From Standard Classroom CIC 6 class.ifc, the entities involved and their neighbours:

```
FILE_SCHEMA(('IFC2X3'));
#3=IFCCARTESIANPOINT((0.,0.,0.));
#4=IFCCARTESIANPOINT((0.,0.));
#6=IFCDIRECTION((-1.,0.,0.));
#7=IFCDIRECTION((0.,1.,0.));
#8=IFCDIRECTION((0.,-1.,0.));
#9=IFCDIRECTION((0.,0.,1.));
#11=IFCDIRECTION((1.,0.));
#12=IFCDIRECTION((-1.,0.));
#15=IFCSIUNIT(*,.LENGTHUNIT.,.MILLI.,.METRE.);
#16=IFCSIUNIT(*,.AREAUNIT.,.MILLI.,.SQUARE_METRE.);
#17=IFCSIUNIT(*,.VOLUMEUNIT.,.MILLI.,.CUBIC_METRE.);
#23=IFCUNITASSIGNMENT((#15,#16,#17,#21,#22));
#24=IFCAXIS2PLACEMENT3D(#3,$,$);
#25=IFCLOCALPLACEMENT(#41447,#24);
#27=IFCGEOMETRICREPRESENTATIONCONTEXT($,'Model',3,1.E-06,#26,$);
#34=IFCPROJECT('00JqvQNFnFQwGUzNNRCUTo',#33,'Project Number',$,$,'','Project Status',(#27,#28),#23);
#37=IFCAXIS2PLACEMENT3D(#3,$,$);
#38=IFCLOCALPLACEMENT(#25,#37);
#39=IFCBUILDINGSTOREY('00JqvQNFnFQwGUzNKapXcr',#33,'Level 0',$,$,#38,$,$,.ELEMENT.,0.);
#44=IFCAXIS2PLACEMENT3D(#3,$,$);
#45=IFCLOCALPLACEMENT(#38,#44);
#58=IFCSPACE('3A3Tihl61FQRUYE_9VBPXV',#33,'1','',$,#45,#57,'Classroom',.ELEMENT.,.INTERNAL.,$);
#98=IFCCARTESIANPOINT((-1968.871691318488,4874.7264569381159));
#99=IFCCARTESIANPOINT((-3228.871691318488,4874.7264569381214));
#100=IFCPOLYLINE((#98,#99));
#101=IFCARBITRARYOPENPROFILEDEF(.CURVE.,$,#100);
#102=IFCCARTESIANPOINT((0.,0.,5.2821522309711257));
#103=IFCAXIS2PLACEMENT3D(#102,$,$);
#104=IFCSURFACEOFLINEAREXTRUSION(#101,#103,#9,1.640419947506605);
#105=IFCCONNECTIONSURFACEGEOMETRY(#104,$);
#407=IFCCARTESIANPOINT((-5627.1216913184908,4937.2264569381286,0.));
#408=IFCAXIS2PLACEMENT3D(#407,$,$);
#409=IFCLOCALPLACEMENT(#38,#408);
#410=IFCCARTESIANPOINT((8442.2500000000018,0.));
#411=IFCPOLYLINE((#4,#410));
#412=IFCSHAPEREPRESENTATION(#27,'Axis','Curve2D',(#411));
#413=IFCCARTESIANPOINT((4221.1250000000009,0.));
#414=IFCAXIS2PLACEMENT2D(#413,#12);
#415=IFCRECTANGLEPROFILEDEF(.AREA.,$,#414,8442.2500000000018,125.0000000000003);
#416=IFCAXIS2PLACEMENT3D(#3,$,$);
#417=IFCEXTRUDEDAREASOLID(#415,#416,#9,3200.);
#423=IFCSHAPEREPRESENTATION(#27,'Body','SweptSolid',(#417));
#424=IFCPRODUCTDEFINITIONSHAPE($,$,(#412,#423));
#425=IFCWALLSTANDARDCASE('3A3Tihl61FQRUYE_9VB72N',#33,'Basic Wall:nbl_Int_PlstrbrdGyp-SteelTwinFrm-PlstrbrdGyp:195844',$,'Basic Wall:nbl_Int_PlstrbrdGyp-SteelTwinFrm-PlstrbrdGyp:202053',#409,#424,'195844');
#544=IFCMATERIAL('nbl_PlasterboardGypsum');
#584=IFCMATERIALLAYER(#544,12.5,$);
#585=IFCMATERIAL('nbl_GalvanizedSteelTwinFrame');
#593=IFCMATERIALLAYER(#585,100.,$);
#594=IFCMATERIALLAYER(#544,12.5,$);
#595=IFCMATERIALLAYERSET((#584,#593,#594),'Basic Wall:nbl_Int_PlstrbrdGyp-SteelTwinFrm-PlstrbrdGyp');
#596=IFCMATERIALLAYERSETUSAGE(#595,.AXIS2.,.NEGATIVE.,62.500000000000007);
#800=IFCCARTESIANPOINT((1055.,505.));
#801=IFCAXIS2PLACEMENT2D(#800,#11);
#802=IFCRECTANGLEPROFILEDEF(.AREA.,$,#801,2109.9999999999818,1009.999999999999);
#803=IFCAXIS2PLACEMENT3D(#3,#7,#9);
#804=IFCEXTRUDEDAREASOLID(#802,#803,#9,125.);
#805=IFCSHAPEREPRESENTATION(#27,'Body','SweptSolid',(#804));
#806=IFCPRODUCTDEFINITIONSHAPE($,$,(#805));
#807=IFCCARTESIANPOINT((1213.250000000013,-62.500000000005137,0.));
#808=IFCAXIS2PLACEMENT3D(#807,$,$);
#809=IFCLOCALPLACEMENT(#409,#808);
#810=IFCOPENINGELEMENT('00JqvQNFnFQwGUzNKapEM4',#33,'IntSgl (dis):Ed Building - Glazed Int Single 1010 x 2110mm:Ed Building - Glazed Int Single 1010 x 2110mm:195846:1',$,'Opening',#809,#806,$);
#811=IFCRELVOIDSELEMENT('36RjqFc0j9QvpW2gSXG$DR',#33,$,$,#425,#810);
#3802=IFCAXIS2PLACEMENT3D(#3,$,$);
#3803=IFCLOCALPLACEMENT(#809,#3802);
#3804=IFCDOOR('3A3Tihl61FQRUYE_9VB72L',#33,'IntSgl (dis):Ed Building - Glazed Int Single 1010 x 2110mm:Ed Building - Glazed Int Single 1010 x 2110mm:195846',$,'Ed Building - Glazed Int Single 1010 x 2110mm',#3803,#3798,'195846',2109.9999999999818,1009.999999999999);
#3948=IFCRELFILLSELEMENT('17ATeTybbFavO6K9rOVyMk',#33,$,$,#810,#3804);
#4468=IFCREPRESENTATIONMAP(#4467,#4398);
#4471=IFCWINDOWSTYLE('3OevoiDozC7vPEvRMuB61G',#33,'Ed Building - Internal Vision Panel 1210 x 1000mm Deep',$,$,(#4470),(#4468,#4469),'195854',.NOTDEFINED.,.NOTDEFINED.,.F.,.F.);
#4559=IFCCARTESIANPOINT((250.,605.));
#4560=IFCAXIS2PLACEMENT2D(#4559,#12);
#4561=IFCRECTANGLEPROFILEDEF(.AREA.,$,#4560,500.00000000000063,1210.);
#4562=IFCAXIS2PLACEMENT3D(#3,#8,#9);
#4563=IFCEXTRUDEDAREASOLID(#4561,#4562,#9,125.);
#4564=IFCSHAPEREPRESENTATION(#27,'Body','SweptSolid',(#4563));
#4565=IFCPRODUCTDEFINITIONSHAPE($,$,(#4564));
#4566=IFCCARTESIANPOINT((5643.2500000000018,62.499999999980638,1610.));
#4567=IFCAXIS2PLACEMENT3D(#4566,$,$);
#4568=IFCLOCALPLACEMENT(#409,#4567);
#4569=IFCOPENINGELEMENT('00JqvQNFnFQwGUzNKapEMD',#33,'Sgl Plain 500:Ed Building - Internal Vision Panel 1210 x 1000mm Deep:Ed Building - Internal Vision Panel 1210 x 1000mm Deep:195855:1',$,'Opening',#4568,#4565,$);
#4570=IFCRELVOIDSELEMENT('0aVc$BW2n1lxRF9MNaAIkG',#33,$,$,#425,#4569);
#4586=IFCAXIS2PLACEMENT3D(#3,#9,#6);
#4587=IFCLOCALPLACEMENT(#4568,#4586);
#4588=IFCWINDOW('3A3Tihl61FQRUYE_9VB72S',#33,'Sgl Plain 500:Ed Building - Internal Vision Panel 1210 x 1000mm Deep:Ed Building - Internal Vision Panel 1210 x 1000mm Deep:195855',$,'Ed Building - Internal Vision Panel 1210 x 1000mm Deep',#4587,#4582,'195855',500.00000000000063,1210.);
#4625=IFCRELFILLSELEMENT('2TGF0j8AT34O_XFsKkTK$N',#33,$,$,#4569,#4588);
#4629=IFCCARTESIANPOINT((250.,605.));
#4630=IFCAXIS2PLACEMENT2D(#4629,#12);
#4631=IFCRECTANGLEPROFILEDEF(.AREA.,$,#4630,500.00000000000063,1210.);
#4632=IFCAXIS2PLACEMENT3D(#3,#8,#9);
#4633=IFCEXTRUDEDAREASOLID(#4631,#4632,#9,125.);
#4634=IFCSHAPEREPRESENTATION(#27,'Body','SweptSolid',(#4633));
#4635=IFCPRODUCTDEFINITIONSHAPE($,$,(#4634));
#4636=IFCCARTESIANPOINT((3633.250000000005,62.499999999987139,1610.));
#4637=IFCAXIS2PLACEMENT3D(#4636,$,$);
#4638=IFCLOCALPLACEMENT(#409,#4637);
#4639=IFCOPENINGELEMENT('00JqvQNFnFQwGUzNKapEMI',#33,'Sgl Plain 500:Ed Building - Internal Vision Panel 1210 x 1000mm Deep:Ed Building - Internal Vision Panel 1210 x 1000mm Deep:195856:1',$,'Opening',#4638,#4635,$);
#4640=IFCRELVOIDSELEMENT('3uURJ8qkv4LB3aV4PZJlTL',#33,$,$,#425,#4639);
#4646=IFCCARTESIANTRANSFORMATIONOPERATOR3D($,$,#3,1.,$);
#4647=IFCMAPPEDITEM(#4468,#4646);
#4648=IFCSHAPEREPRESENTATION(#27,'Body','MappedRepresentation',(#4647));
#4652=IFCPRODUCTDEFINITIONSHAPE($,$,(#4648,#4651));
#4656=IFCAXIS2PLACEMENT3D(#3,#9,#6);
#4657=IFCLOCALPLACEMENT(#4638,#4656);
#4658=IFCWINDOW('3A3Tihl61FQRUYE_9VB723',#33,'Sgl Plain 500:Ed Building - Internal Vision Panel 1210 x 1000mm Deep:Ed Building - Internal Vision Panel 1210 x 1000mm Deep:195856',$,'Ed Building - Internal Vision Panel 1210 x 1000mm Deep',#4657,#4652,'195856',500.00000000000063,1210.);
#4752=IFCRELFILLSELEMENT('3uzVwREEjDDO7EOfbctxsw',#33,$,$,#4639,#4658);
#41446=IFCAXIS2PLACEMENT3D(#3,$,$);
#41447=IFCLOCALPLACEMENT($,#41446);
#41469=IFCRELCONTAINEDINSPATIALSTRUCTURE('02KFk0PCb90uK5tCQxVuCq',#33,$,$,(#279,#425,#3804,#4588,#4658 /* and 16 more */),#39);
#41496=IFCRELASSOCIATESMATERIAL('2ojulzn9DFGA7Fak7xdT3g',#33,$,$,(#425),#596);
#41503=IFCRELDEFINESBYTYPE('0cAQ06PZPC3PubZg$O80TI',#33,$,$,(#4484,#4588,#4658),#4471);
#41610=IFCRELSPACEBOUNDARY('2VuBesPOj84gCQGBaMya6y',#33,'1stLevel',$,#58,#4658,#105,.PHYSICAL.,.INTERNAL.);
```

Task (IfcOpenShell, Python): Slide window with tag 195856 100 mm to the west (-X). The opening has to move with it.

```python
import numpy as np
import ifcopenshell
import ifcopenshell.api.geometry
import ifcopenshell.util.placement
import ifcopenshell.util.unit

model = ifcopenshell.open("Standard Classroom CIC 6 class.ifc")
unit_scale = ifcopenshell.util.unit.calculate_unit_scale(model)

window = model.by_id(4658)
opening = window.FillsVoids[0].RelatingOpeningElement
wall = opening.VoidsElements[0].RelatingBuildingElement

wall_matrix = ifcopenshell.util.placement.get_local_placement(wall.ObjectPlacement)
shift = wall_matrix[:3, 0] * -0.1 / unit_scale
before = ifcopenshell.util.placement.get_local_placement(window.ObjectPlacement)[:3, 3].copy()

# The window is placed relative to its opening, so it follows when the opening moves.
matrix = ifcopenshell.util.placement.get_local_placement(opening.ObjectPlacement)
matrix[:3, 3] += shift
ifcopenshell.api.geometry.edit_object_placement(
    model, product=opening, matrix=matrix, is_si=False, should_transform_children=True
)

# Space boundary surfaces are stored in each space's coordinates; move them too.
for rel in window.ProvidesBoundaries:
    if not rel.ConnectionGeometry:
        continue
    surface = rel.ConnectionGeometry.SurfaceOnRelatingElement
    space_matrix = ifcopenshell.util.placement.get_local_placement(rel.RelatingSpace.ObjectPlacement)
    point = np.array(surface.Position.Location.Coordinates) + space_matrix[:3, :3].T @ shift
    surface.Position = model.createIfcAxis2Placement3D(
        model.createIfcCartesianPoint(point.tolist()), surface.Position.Axis, surface.Position.RefDirection
    )

after = ifcopenshell.util.placement.get_local_placement(window.ObjectPlacement)[:3, 3]
print("window moved by", (after - before).round(3) + 0.0)

model.write("Standard Classroom CIC 6 class_updated.ifc")
```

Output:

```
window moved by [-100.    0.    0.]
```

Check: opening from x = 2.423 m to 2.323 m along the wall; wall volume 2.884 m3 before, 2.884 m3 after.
